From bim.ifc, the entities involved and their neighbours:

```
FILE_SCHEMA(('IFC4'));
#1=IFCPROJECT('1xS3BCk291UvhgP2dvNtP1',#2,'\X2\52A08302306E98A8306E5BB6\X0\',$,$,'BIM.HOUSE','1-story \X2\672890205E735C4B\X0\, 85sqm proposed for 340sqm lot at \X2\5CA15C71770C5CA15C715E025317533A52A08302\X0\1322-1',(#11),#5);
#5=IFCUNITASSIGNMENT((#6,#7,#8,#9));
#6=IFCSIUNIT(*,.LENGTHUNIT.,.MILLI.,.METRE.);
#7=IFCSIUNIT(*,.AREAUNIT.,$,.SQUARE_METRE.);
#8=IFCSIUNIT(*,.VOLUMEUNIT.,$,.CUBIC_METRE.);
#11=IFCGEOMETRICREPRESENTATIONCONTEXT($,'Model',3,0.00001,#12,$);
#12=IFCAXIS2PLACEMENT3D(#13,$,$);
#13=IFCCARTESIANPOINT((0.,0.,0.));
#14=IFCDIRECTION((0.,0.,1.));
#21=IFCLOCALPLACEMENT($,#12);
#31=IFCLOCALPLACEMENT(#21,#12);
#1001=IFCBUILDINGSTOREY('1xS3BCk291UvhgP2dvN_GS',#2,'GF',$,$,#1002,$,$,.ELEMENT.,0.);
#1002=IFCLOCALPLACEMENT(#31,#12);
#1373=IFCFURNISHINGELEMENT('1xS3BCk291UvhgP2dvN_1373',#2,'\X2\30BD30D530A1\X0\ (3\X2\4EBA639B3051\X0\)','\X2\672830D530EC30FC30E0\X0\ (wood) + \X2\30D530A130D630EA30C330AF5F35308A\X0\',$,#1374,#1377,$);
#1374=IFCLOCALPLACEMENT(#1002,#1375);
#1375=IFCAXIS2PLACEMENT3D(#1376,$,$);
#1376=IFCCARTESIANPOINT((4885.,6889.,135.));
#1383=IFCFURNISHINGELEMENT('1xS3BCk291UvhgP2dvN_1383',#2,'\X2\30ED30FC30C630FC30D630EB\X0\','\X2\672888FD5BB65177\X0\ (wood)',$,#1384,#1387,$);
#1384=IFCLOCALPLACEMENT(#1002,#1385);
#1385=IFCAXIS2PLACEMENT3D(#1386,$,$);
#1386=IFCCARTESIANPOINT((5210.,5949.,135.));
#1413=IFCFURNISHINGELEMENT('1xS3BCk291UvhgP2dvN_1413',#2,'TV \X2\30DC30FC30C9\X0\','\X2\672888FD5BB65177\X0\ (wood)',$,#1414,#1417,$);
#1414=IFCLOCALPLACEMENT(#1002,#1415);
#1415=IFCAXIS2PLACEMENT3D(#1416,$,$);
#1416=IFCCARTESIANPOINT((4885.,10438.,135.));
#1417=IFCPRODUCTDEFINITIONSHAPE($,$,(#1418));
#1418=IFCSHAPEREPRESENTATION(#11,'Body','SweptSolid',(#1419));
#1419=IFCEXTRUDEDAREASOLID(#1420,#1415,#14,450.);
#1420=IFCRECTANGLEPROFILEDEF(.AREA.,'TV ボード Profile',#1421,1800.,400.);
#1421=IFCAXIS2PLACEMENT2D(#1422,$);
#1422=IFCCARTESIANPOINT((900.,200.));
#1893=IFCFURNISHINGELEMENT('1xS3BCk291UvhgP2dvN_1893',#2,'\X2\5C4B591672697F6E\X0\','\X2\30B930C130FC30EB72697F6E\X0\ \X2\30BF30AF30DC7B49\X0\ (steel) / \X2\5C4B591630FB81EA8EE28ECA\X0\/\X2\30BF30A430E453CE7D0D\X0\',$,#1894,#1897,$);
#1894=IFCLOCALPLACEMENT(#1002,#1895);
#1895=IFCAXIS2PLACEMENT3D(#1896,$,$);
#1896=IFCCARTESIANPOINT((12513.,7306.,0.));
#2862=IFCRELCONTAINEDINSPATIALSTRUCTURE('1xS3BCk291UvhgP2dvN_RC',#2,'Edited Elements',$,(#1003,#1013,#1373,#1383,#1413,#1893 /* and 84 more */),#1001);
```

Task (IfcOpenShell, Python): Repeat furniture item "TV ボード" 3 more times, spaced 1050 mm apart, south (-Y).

```python
import numpy as np
import ifcopenshell
import ifcopenshell.api.geometry
import ifcopenshell.api.root
import ifcopenshell.util.element
import ifcopenshell.util.placement
import ifcopenshell.util.unit

model = ifcopenshell.open("bim.ifc")
unit_scale = ifcopenshell.util.unit.calculate_unit_scale(model)


def reuse_history(source, copy):
    """copy_class also copies each property set's owner history, people and application; keep the originals."""
    for rel in copy.IsDefinedBy:
        if rel.is_a("IfcRelDefinesByProperties") and (history := rel.RelatingPropertyDefinition.OwnerHistory):
            rel.RelatingPropertyDefinition.OwnerHistory = source.OwnerHistory
            ifcopenshell.util.element.remove_deep2(model, history)


source = model.by_guid("1xS3BCk291UvhgP2dvN_1413")
base = ifcopenshell.util.placement.get_local_placement(source.ObjectPlacement)
step = np.array([0.0, -1.0, 0.0]) * 1.05 / unit_scale

for i in range(1, 4):
    copy = ifcopenshell.api.root.copy_class(model, product=source)
    copy.Representation = ifcopenshell.util.element.copy_deep(
        model, source.Representation, exclude=["IfcGeometricRepresentationContext", "IfcRepresentationMap"]
    )
    reuse_history(source, copy)
    matrix = base.copy()
    matrix[:3, 3] += i * step
    print("added at", matrix[:3, 3].round(3) + 0.0)
    ifcopenshell.api.geometry.edit_object_placement(model, product=copy, matrix=matrix, is_si=False)

model.write("bim_v2.ifc")
```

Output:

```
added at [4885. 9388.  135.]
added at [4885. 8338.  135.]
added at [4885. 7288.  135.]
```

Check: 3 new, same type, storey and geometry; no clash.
